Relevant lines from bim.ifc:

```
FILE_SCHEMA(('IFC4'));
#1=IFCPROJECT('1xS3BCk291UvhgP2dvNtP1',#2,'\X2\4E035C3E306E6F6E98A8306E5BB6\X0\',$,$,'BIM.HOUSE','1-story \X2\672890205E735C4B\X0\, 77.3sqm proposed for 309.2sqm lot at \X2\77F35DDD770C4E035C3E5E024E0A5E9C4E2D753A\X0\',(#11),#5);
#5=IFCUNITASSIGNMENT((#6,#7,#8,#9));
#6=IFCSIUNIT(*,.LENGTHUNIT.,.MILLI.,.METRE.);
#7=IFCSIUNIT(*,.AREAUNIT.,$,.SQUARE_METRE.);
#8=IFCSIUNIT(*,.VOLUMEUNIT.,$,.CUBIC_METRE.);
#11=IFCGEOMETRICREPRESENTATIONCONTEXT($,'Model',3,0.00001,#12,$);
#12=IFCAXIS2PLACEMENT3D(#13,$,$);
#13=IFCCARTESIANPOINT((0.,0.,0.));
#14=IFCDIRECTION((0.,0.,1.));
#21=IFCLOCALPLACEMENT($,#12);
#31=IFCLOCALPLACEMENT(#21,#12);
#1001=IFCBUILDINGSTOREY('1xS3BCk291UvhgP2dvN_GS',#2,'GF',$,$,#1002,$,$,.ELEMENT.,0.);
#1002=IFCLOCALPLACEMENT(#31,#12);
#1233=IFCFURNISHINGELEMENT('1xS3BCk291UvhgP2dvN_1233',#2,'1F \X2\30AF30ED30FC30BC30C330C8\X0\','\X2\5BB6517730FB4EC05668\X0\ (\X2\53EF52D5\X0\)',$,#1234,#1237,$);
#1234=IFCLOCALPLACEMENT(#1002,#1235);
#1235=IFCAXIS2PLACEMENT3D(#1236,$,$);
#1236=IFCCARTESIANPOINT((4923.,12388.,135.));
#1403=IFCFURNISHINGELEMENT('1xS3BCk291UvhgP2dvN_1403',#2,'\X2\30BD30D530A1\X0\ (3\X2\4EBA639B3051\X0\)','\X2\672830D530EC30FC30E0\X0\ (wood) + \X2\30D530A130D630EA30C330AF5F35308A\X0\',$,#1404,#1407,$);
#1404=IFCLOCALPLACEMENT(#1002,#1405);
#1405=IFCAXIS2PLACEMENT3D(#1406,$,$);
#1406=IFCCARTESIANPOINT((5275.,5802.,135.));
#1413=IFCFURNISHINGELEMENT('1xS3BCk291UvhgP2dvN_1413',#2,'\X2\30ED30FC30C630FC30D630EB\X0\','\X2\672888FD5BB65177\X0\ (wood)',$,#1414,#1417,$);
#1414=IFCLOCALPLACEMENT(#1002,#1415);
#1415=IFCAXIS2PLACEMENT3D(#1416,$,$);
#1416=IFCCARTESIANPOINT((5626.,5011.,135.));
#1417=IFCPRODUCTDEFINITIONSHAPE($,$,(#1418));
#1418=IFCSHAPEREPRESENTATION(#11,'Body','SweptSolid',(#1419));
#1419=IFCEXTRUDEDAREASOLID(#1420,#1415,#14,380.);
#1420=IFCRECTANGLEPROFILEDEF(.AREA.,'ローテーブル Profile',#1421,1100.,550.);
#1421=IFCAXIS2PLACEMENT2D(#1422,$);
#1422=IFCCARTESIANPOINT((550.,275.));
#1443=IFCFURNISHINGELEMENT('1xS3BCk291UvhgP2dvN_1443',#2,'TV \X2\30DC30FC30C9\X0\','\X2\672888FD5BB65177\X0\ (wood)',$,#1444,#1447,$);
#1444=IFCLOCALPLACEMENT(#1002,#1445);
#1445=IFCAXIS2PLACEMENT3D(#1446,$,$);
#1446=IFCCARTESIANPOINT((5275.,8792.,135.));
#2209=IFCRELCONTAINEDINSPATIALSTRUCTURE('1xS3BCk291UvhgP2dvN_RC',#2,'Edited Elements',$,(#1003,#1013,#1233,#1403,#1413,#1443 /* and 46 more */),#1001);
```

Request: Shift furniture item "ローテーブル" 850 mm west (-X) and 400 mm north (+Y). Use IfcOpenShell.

```python
import ifcopenshell
import ifcopenshell.api.geometry
import ifcopenshell.util.placement
import ifcopenshell.util.unit

model = ifcopenshell.open("bim.ifc")
unit_scale = ifcopenshell.util.unit.calculate_unit_scale(model)

item = model.by_id(1413)
matrix = ifcopenshell.util.placement.get_local_placement(item.ObjectPlacement)
matrix[0, 3] -= 0.85 / unit_scale
matrix[1, 3] += 0.4 / unit_scale
ifcopenshell.api.geometry.edit_object_placement(model, product=item, matrix=matrix, is_si=False)

print(ifcopenshell.util.placement.get_local_placement(item.ObjectPlacement).round(3) + 0.0)

model.write("bim_rev.ifc")
```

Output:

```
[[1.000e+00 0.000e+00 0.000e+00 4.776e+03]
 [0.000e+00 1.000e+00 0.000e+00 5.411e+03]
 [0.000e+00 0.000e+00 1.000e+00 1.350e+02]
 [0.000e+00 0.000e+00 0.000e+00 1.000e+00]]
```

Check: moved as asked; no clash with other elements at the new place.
